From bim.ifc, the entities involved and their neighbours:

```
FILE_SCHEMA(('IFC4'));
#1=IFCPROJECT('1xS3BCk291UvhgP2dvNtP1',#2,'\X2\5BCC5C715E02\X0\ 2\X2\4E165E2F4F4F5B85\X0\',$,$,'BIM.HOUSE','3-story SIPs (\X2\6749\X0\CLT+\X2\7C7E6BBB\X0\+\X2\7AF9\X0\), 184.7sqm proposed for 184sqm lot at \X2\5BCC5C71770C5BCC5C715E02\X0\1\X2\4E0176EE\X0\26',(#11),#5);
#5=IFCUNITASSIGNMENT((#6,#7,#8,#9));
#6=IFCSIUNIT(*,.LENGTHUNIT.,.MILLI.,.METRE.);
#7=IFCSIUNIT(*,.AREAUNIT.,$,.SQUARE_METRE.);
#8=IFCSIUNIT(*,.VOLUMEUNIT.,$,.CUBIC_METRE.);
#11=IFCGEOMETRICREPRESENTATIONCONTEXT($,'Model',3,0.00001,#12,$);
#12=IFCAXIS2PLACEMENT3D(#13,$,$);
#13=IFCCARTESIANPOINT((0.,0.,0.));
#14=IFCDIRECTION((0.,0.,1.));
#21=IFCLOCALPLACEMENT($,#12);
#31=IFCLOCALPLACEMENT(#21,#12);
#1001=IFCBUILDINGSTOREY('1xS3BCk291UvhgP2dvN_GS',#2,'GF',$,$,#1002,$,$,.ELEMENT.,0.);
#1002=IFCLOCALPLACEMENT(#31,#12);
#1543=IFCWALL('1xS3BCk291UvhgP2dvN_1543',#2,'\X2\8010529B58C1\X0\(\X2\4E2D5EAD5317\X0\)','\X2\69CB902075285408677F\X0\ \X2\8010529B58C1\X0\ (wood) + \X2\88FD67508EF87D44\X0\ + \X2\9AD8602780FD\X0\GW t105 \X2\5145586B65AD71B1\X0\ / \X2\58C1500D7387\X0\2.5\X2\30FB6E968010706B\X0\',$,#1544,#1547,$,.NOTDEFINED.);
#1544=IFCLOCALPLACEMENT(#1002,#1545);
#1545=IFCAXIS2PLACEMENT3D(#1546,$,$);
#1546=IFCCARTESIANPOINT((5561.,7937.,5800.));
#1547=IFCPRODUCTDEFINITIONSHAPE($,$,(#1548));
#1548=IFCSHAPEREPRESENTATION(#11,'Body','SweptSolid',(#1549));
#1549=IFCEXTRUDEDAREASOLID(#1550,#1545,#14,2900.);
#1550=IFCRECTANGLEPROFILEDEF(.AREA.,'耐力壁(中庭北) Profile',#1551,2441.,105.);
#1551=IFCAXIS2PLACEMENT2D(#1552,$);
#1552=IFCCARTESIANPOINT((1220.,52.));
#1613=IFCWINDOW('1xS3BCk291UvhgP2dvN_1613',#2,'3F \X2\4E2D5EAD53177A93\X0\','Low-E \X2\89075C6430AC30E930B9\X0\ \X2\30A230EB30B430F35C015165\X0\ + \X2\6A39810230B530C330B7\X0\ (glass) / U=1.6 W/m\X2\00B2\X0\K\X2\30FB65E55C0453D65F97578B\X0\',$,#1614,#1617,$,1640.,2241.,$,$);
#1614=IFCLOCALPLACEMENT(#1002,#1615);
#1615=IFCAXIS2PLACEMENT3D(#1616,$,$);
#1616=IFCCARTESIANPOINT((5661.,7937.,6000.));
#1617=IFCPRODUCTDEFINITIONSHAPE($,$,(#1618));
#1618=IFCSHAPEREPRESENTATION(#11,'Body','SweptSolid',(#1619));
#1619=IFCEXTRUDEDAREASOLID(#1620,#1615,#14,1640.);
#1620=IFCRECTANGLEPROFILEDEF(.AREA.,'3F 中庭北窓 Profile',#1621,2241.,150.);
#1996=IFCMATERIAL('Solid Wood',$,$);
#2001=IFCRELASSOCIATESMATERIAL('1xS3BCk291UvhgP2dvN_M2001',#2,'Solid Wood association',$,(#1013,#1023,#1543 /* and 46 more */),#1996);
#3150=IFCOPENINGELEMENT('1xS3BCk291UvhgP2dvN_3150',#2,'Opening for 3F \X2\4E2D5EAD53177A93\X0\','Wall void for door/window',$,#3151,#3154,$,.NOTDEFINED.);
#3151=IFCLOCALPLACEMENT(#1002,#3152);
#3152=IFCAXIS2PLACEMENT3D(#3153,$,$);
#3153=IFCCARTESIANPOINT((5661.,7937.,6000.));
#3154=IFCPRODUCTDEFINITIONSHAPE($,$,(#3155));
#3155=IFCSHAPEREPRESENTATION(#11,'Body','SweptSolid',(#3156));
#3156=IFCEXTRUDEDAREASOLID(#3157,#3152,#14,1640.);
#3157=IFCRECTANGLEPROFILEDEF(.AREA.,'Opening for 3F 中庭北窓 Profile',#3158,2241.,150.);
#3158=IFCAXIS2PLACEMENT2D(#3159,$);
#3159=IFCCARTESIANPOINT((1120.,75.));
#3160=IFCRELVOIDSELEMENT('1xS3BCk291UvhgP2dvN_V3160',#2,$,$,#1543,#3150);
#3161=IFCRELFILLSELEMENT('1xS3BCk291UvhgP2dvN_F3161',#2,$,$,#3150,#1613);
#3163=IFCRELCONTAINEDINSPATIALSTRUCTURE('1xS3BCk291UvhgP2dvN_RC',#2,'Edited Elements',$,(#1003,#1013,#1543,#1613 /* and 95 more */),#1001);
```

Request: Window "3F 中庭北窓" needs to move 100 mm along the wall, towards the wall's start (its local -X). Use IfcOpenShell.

```python
import ifcopenshell
import ifcopenshell.api.geometry
import ifcopenshell.util.placement

model = ifcopenshell.open("bim.ifc")

window = model.by_guid("1xS3BCk291UvhgP2dvN_1613")
opening = window.FillsVoids[0].RelatingOpeningElement
wall = opening.VoidsElements[0].RelatingBuildingElement

wall_matrix = ifcopenshell.util.placement.get_local_placement(wall.ObjectPlacement)
shift = wall_matrix[:3, 0] * -100.0
before = ifcopenshell.util.placement.get_local_placement(window.ObjectPlacement)[:3, 3].copy()

# The window is not placed relative to its opening, so move both.
for product in (opening, window):
    matrix = ifcopenshell.util.placement.get_local_placement(product.ObjectPlacement)
    matrix[:3, 3] += shift
    ifcopenshell.api.geometry.edit_object_placement(model, product=product, matrix=matrix, is_si=False)

after = ifcopenshell.util.placement.get_local_placement(window.ObjectPlacement)[:3, 3]
print("window moved by", (after - before).round(3) + 0.0)

model.write("bim_updated.ifc")
```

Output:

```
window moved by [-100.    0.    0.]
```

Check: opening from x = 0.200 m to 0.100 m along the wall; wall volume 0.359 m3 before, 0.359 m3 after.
